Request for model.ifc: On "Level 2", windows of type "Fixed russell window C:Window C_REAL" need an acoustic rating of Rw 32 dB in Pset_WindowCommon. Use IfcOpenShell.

First a look at what the model holds.

```python
import ifcopenshell
import ifcopenshell.util.element

model = ifcopenshell.open("model.ifc")
print(model.schema)
storey = next(s for s in model.by_type("IfcBuildingStorey") if s.Name == "Level 2")
windows = [e for e in ifcopenshell.util.element.get_decomposition(storey) if e.is_a("IfcWindow")]
seen = {}
for e in windows:
    element_type = ifcopenshell.util.element.get_type(e)
    key = (element_type.Name if element_type != e and element_type else None, ifcopenshell.util.element.get_pset(e, "Pset_WindowCommon", "AcousticRating"))
    seen[key] = seen.get(key, 0) + 1
for (name, value), count in sorted(seen.items(), key=str):
    print(count, "x", name, "|", value)
```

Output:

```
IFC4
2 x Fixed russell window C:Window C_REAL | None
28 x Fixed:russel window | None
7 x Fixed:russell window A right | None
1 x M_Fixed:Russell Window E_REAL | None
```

```python
import ifcopenshell
import ifcopenshell.api.pset
import ifcopenshell.util.element

model = ifcopenshell.open("model.ifc")

storey = next(s for s in model.by_type("IfcBuildingStorey") if s.Name == "Level 2")
windows = [e for e in ifcopenshell.util.element.get_decomposition(storey) if e.is_a("IfcWindow")]

count = 0
for e in windows:
    element_type = ifcopenshell.util.element.get_type(e)
    if element_type in (None, e) or element_type.Name != "Fixed russell window C:Window C_REAL":
        continue
    # add_pset returns the element's existing set when there is one.
    pset = ifcopenshell.api.pset.add_pset(model, product=e, name="Pset_WindowCommon")
    ifcopenshell.api.pset.edit_pset(model, pset=pset, properties={"AcousticRating": "Rw 32 dB"})
    count += 1

print(count, "windows updated")

model.write("model_edited.ifc")
```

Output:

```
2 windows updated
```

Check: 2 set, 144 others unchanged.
